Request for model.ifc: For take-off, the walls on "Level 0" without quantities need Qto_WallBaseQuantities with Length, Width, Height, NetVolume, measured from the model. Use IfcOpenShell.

First a look at what the model holds.

```python
import ifcopenshell
import ifcopenshell.util.element
import ifcopenshell.util.unit

model = ifcopenshell.open("model.ifc")
print(model.schema)
for unit_type in ("LENGTHUNIT", "AREAUNIT", "VOLUMEUNIT"):
    print(unit_type, ifcopenshell.util.unit.calculate_unit_scale(model, unit_type))
storey = next(s for s in model.by_type("IfcBuildingStorey") if s.Name == "Level 0")
walls = [e for e in ifcopenshell.util.element.get_decomposition(storey) if e.is_a("IfcWall")]
for e in sorted(walls, key=lambda e: e.id()):
    print(e.id(), e.is_a(), e.Name, list(ifcopenshell.util.element.get_psets(e, qtos_only=True)), sep=" | ")
```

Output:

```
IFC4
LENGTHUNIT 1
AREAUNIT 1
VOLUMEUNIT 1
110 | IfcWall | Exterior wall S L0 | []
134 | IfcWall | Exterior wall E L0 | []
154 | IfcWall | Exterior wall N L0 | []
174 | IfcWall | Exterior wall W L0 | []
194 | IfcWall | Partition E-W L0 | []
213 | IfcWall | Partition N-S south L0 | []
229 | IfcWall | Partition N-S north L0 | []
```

```python
import ifcopenshell
import ifcopenshell.api.pset
import ifcopenshell.geom
import ifcopenshell.util.element
import ifcopenshell.util.shape
import ifcopenshell.util.unit

model = ifcopenshell.open("model.ifc")
unit_scale = ifcopenshell.util.unit.calculate_unit_scale(model)
volume_scale = ifcopenshell.util.unit.calculate_unit_scale(model, "VOLUMEUNIT")
settings = ifcopenshell.geom.settings()

storey = next(s for s in model.by_type("IfcBuildingStorey") if s.Name == "Level 0")
walls = [e for e in ifcopenshell.util.element.get_decomposition(storey) if e.is_a("IfcWall")]

for e in sorted(walls, key=lambda e: e.id()):
    if ifcopenshell.util.element.get_psets(e, qtos_only=True, should_inherit=False):
        continue
    # Geometry comes back in metres, in the element's own axes.
    shape = ifcopenshell.geom.create_shape(settings, e)
    values = {
        "Length": ifcopenshell.util.shape.get_x(shape.geometry) / unit_scale,
        "Width": ifcopenshell.util.shape.get_y(shape.geometry) / unit_scale,
        "Height": ifcopenshell.util.shape.get_z(shape.geometry) / unit_scale,
        "NetVolume": ifcopenshell.util.shape.get_volume(shape.geometry) / volume_scale,
    }
    qto = ifcopenshell.api.pset.add_qto(model, product=e, name="Qto_WallBaseQuantities")
    ifcopenshell.api.pset.edit_qto(model, qto=qto, properties=values)
    print(e.id(), {k: round(v, 3) for k, v in values.items()})

model.write("model_v2.ifc")
```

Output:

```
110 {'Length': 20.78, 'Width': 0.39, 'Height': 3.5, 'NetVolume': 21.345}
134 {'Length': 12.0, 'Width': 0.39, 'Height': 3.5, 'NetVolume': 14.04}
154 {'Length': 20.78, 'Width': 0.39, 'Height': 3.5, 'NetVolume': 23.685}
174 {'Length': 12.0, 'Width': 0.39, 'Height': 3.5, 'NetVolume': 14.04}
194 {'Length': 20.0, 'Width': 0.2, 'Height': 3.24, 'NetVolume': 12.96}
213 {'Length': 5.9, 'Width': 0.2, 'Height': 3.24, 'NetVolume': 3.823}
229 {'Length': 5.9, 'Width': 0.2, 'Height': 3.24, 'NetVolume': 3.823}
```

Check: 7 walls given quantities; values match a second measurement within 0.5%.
